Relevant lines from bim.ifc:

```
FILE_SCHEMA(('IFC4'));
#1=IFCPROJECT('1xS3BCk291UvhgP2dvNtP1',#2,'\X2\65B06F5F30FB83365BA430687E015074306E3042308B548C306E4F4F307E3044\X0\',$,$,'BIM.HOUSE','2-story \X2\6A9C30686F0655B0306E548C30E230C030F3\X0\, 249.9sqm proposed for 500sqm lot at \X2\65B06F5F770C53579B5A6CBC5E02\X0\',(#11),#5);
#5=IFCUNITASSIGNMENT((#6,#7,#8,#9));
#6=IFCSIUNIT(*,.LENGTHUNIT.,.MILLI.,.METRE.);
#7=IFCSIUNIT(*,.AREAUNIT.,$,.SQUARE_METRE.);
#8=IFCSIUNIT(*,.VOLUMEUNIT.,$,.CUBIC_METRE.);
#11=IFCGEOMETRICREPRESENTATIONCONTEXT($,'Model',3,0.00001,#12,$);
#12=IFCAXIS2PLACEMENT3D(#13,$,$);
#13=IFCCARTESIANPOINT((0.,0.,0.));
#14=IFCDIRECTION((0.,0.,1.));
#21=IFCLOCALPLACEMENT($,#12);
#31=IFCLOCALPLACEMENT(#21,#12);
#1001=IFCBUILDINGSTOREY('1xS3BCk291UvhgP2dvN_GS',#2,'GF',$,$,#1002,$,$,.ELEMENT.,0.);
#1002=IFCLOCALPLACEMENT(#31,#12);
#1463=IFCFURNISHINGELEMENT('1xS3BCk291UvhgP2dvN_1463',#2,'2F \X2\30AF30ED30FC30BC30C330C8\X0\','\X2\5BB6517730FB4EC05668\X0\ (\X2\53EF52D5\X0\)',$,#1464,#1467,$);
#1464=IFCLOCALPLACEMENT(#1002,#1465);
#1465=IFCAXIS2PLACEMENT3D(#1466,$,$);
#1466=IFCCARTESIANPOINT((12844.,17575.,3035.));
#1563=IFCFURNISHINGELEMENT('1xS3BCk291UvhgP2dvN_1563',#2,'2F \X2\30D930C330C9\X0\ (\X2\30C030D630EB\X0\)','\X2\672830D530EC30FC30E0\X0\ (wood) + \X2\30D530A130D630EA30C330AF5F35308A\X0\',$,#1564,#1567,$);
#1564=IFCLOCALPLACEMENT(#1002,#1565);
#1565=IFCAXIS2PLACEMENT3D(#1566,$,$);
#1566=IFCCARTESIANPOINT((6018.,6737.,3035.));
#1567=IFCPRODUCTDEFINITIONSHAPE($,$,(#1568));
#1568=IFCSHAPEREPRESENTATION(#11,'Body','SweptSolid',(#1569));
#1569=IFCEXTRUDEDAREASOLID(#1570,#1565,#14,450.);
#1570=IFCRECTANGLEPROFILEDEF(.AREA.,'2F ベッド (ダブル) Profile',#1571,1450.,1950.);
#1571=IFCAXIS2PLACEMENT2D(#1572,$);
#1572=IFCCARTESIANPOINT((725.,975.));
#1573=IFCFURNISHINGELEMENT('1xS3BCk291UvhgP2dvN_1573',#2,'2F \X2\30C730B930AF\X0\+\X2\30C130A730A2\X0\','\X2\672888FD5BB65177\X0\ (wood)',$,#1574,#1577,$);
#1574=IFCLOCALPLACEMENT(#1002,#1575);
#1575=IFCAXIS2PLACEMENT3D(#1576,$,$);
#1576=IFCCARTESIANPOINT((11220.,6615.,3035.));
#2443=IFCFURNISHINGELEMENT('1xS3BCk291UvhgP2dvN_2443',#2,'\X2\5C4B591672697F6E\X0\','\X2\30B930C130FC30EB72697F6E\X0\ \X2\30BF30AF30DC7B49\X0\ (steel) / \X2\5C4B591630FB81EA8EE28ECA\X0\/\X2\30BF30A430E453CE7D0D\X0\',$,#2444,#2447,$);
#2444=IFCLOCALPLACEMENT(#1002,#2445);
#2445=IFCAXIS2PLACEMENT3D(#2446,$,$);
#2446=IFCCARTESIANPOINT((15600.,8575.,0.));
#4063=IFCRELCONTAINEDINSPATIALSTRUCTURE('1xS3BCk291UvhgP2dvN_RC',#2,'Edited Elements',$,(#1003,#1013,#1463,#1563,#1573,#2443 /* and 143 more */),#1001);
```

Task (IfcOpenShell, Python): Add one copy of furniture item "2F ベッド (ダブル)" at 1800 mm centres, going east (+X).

```python
import numpy as np
import ifcopenshell
import ifcopenshell.api.geometry
import ifcopenshell.api.root
import ifcopenshell.util.element
import ifcopenshell.util.placement

model = ifcopenshell.open("bim.ifc")


def reuse_history(source, copy):
    """copy_class also copies each property set's owner history, people and application; keep the originals."""
    for rel in copy.IsDefinedBy:
        if rel.is_a("IfcRelDefinesByProperties") and (history := rel.RelatingPropertyDefinition.OwnerHistory):
            rel.RelatingPropertyDefinition.OwnerHistory = source.OwnerHistory
            ifcopenshell.util.element.remove_deep2(model, history)


source = model.by_guid("1xS3BCk291UvhgP2dvN_1563")
base = ifcopenshell.util.placement.get_local_placement(source.ObjectPlacement)
step = np.array([1.0, 0.0, 0.0]) * 1800.0

for i in range(1, 2):
    copy = ifcopenshell.api.root.copy_class(model, product=source)
    copy.Representation = ifcopenshell.util.element.copy_deep(
        model, source.Representation, exclude=["IfcGeometricRepresentationContext", "IfcRepresentationMap"]
    )
    reuse_history(source, copy)
    matrix = base.copy()
    matrix[:3, 3] += i * step
    print("added at", matrix[:3, 3].round(3) + 0.0)
    ifcopenshell.api.geometry.edit_object_placement(model, product=copy, matrix=matrix, is_si=False)

model.write("bim_updated.ifc")
```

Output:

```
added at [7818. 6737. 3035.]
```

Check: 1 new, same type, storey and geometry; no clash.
